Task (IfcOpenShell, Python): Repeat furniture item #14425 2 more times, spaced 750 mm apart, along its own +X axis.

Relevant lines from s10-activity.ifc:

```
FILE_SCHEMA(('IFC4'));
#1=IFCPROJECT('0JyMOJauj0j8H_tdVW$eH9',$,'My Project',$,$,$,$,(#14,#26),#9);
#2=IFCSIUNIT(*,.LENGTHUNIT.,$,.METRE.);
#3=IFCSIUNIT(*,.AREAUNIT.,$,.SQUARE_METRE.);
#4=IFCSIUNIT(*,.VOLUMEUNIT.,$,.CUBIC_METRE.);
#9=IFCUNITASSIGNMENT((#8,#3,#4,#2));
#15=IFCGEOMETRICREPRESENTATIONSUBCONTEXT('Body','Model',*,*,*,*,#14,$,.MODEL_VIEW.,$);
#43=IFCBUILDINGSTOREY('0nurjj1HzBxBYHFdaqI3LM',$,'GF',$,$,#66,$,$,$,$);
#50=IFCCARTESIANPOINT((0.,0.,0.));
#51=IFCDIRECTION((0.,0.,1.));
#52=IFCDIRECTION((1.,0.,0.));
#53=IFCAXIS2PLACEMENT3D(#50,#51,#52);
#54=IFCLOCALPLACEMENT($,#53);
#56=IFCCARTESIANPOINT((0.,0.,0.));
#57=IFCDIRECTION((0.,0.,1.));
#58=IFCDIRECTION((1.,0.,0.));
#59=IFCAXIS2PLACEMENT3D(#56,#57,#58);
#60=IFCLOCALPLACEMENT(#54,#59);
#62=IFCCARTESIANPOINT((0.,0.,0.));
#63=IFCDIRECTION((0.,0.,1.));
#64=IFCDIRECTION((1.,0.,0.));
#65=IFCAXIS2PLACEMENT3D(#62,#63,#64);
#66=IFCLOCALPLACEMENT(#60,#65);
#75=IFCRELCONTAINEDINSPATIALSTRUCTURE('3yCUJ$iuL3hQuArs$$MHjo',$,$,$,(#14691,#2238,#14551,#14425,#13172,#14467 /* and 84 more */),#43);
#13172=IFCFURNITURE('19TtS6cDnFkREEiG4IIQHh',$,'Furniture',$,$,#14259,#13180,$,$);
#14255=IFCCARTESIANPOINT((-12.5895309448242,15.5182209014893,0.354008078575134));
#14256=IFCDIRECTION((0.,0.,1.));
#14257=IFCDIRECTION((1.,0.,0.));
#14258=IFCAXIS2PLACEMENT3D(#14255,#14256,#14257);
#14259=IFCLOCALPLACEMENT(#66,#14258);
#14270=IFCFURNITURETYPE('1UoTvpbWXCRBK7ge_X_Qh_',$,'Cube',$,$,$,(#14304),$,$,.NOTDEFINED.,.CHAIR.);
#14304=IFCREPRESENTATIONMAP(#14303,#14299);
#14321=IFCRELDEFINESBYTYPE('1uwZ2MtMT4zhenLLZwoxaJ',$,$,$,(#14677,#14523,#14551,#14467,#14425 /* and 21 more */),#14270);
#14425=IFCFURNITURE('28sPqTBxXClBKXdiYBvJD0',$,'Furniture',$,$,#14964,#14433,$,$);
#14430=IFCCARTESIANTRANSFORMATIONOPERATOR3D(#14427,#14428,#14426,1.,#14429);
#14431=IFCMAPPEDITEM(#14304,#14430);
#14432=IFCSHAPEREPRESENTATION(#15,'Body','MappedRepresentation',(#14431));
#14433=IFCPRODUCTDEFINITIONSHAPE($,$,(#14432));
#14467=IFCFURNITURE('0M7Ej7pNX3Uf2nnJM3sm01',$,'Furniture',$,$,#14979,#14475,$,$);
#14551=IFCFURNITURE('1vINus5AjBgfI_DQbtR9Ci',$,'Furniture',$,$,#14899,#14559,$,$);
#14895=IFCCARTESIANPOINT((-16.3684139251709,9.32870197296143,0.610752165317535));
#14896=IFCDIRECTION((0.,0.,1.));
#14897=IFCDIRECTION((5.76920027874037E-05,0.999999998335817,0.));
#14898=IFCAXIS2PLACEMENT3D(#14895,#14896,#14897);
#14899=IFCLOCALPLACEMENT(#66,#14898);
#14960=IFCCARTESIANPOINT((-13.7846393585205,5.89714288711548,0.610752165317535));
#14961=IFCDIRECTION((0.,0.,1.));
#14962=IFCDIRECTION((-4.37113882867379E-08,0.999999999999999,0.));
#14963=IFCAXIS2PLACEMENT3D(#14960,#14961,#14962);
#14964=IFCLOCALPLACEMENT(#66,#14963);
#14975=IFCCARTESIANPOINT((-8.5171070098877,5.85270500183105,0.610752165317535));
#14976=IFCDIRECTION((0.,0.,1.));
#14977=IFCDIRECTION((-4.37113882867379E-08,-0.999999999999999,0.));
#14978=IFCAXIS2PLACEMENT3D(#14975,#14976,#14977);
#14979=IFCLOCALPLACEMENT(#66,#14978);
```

```python
import ifcopenshell
import ifcopenshell.api.geometry
import ifcopenshell.api.root
import ifcopenshell.util.element
import ifcopenshell.util.placement
import ifcopenshell.util.unit

model = ifcopenshell.open("s10-activity.ifc")
unit_scale = ifcopenshell.util.unit.calculate_unit_scale(model)

source = model.by_id(14425)
base = ifcopenshell.util.placement.get_local_placement(source.ObjectPlacement)
step = base[:3, 0] * 0.75 / unit_scale

for i in range(1, 3):
    copy = ifcopenshell.api.root.copy_class(model, product=source)
    copy.Representation = ifcopenshell.util.element.copy_deep(
        model, source.Representation, exclude=["IfcGeometricRepresentationContext", "IfcRepresentationMap"]
    )
    matrix = base.copy()
    matrix[:3, 3] += i * step
    print("added at", matrix[:3, 3].round(3) + 0.0)
    ifcopenshell.api.geometry.edit_object_placement(model, product=copy, matrix=matrix, is_si=False)

model.write("s10-activity_updated.ifc")
```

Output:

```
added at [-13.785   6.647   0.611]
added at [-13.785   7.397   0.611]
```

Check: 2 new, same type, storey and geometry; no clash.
